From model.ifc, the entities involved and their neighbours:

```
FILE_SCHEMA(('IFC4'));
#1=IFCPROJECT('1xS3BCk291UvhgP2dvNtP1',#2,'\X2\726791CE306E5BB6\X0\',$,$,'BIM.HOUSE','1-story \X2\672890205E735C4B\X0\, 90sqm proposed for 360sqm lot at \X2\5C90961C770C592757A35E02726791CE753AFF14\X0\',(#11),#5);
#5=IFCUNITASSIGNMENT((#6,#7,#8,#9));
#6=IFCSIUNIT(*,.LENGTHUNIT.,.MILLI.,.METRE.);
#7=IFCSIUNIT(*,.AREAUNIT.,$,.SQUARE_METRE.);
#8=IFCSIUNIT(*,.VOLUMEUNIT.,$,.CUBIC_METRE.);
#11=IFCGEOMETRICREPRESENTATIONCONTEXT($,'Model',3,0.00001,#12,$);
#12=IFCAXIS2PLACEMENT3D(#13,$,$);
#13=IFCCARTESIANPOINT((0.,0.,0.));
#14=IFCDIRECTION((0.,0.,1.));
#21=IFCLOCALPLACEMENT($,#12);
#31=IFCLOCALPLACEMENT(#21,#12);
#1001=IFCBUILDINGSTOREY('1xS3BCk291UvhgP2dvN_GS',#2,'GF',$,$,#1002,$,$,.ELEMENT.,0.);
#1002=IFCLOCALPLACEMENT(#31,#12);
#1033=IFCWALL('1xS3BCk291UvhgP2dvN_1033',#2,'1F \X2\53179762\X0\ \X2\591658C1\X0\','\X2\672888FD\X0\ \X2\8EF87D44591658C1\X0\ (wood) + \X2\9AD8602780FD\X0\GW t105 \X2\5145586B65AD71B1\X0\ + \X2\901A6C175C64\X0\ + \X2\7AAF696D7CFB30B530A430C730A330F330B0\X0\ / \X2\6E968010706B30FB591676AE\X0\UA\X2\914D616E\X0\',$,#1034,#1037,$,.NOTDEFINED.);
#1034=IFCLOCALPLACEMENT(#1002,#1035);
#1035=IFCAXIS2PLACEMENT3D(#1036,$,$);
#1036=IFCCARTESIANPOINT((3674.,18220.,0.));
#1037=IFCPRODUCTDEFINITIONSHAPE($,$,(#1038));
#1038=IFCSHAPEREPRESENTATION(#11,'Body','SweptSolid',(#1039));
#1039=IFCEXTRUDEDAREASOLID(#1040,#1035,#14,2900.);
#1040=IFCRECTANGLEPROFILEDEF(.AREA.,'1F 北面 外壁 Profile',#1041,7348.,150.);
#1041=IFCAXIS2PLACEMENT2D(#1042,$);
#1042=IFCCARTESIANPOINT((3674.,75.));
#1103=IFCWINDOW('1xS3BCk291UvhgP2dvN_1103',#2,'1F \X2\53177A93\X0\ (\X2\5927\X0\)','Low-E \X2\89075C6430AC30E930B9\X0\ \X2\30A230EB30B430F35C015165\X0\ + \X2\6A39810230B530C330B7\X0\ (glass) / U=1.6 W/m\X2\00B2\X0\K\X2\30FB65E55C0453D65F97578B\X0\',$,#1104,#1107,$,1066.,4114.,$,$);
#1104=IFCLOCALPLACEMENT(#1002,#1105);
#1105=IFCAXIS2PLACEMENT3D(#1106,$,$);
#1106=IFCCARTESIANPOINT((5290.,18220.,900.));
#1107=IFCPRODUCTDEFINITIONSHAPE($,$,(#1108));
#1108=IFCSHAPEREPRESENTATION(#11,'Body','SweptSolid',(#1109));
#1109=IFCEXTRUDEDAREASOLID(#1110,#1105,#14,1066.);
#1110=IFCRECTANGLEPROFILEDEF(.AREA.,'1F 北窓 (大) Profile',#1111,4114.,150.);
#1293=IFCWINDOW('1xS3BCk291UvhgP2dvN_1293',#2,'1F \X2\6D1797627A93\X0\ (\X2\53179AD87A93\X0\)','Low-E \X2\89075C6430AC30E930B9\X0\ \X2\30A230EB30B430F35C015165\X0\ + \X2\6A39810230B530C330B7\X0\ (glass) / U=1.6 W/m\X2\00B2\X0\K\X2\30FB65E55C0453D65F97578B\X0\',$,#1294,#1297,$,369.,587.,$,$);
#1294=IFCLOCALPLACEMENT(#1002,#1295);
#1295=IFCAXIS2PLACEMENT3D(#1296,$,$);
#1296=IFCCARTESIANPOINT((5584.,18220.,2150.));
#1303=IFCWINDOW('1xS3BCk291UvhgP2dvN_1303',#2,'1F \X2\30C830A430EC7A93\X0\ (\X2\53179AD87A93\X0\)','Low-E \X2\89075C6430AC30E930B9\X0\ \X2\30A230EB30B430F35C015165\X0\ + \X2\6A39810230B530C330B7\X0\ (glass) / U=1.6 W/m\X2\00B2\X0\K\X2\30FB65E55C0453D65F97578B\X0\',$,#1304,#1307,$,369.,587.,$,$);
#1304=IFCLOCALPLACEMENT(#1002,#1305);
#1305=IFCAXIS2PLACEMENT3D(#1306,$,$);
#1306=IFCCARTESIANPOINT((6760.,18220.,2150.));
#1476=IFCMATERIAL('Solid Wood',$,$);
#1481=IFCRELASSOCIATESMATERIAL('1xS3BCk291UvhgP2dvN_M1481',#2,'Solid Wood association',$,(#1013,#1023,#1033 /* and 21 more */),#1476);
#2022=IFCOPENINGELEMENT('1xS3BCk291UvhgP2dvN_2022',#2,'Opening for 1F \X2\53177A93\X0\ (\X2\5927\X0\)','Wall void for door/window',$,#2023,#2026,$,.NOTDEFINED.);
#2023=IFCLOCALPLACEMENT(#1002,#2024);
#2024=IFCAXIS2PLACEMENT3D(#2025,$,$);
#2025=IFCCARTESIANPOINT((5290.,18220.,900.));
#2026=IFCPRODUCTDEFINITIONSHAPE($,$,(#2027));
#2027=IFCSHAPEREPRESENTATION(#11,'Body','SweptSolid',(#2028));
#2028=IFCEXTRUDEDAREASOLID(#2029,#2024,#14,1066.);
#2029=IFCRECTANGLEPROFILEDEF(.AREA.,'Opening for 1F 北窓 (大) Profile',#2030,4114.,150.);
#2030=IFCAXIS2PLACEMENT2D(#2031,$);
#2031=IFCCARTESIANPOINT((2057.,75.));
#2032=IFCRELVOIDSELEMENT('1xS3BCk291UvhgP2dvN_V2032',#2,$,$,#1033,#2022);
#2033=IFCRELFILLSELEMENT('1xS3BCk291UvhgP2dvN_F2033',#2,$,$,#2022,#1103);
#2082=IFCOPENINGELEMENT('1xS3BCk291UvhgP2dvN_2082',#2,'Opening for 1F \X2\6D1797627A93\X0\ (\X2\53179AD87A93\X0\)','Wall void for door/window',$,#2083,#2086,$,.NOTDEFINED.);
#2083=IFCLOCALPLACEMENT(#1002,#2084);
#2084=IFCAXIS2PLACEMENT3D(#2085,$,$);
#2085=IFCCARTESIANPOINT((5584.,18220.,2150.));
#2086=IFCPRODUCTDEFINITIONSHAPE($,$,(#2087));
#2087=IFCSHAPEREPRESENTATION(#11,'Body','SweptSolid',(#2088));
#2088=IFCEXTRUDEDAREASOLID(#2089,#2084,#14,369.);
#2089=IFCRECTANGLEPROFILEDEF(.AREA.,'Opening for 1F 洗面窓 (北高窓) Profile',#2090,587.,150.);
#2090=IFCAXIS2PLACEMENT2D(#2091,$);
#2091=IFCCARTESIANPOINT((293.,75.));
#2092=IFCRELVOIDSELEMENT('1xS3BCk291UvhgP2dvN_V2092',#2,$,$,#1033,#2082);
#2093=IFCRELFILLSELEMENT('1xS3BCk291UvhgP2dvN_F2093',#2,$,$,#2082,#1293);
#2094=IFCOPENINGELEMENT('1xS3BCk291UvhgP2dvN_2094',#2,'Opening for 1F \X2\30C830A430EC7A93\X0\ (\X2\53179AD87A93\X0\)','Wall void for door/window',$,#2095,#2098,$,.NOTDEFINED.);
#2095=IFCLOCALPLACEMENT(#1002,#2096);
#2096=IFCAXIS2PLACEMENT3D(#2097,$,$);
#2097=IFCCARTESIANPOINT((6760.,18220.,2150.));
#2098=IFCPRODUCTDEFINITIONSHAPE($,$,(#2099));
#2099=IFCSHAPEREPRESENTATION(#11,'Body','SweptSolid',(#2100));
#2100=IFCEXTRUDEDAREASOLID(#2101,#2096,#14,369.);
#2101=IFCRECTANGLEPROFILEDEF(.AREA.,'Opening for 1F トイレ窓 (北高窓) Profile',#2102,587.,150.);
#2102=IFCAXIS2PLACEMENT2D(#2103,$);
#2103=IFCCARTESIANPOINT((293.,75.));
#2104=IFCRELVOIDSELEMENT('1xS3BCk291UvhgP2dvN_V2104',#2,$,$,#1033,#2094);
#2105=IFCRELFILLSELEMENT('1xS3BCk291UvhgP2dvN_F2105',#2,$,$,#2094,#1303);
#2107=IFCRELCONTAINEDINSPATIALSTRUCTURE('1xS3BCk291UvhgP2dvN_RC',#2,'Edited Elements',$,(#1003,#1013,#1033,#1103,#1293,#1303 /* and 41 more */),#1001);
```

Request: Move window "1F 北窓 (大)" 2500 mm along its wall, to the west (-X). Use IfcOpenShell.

```python
import ifcopenshell
import ifcopenshell.api.geometry
import ifcopenshell.util.placement
import ifcopenshell.util.unit

model = ifcopenshell.open("model.ifc")
unit_scale = ifcopenshell.util.unit.calculate_unit_scale(model)

window = model.by_id(1103)
opening = window.FillsVoids[0].RelatingOpeningElement
wall = opening.VoidsElements[0].RelatingBuildingElement

wall_matrix = ifcopenshell.util.placement.get_local_placement(wall.ObjectPlacement)
shift = wall_matrix[:3, 0] * -2.5 / unit_scale
before = ifcopenshell.util.placement.get_local_placement(window.ObjectPlacement)[:3, 3].copy()

# The window is not placed relative to its opening, so move both.
for product in (opening, window):
    matrix = ifcopenshell.util.placement.get_local_placement(product.ObjectPlacement)
    matrix[:3, 3] += shift
    ifcopenshell.api.geometry.edit_object_placement(model, product=product, matrix=matrix, is_si=False)

after = ifcopenshell.util.placement.get_local_placement(window.ObjectPlacement)[:3, 3]
print("window moved by", (after - before).round(3) + 0.0)

model.write("model_edited.ifc")
```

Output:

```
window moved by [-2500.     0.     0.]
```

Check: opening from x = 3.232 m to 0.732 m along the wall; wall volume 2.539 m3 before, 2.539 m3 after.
